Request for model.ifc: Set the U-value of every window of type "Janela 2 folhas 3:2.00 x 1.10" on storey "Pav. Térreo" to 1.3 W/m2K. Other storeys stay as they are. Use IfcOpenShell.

First a look at what the model holds.

```python
import ifcopenshell
import ifcopenshell.util.element

model = ifcopenshell.open("model.ifc")
print(model.schema)
storey = next(s for s in model.by_type("IfcBuildingStorey") if s.Name == "Pav. Térreo")
windows = [e for e in ifcopenshell.util.element.get_decomposition(storey) if e.is_a("IfcWindow")]
seen = {}
for e in windows:
    element_type = ifcopenshell.util.element.get_type(e)
    key = (element_type.Name if element_type != e and element_type else None, ifcopenshell.util.element.get_pset(e, "Pset_WindowCommon", "ThermalTransmittance"))
    seen[key] = seen.get(key, 0) + 1
for (name, value), count in sorted(seen.items(), key=str):
    print(count, "x", name, "|", value)
```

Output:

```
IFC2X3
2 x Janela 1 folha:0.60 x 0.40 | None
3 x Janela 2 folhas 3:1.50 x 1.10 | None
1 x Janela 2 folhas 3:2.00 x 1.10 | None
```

```python
import ifcopenshell
import ifcopenshell.api.pset
import ifcopenshell.util.element

model = ifcopenshell.open("model.ifc")

storey = next(s for s in model.by_type("IfcBuildingStorey") if s.Name == "Pav. Térreo")
windows = [e for e in ifcopenshell.util.element.get_decomposition(storey) if e.is_a("IfcWindow")]

count = 0
for e in windows:
    element_type = ifcopenshell.util.element.get_type(e)
    if element_type in (None, e) or element_type.Name != "Janela 2 folhas 3:2.00 x 1.10":
        continue
    # add_pset returns the element's existing set when there is one.
    pset = ifcopenshell.api.pset.add_pset(model, product=e, name="Pset_WindowCommon")
    ifcopenshell.api.pset.edit_pset(model, pset=pset, properties={"ThermalTransmittance": 1.3})
    count += 1

print(count, "windows updated")

model.write("model_rev.ifc")
```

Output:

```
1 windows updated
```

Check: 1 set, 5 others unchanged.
